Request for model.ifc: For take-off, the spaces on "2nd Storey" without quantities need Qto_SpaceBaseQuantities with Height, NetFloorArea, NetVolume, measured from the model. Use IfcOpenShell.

First a look at what the model holds.

```python
import ifcopenshell
import ifcopenshell.util.element
import ifcopenshell.util.unit

model = ifcopenshell.open("model.ifc")
print(model.schema)
for unit_type in ("LENGTHUNIT", "AREAUNIT", "VOLUMEUNIT"):
    print(unit_type, ifcopenshell.util.unit.calculate_unit_scale(model, unit_type))
storey = next(s for s in model.by_type("IfcBuildingStorey") if s.Name == "2nd Storey")
spaces = [e for e in ifcopenshell.util.element.get_decomposition(storey) if e.is_a("IfcSpace")]
for e in sorted(spaces, key=lambda e: e.id()):
    print(e.id(), e.is_a(), e.Name, list(ifcopenshell.util.element.get_psets(e, qtos_only=True)), sep=" | ")
```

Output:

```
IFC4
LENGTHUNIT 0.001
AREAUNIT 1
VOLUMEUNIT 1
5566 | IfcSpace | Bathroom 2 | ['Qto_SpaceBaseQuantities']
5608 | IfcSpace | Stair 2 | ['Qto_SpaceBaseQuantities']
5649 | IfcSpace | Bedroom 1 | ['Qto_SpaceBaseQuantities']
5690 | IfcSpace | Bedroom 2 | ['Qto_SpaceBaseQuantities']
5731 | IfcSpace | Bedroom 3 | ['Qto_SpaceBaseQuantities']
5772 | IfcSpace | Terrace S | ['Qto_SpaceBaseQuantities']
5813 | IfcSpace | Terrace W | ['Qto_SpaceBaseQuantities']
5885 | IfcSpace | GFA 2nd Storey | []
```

```python
import ifcopenshell
import ifcopenshell.api.pset
import ifcopenshell.geom
import ifcopenshell.util.element
import ifcopenshell.util.shape
import ifcopenshell.util.unit

model = ifcopenshell.open("model.ifc")
unit_scale = ifcopenshell.util.unit.calculate_unit_scale(model)
area_scale = ifcopenshell.util.unit.calculate_unit_scale(model, "AREAUNIT")
volume_scale = ifcopenshell.util.unit.calculate_unit_scale(model, "VOLUMEUNIT")
settings = ifcopenshell.geom.settings()

storey = next(s for s in model.by_type("IfcBuildingStorey") if s.Name == "2nd Storey")
spaces = [e for e in ifcopenshell.util.element.get_decomposition(storey) if e.is_a("IfcSpace")]

for e in sorted(spaces, key=lambda e: e.id()):
    if ifcopenshell.util.element.get_psets(e, qtos_only=True, should_inherit=False):
        continue
    # Geometry comes back in metres, in the element's own axes.
    shape = ifcopenshell.geom.create_shape(settings, e)
    values = {
        "Height": ifcopenshell.util.shape.get_z(shape.geometry) / unit_scale,
        "NetFloorArea": ifcopenshell.util.shape.get_footprint_area(shape.geometry) / area_scale,
        "NetVolume": ifcopenshell.util.shape.get_volume(shape.geometry) / volume_scale,
    }
    qto = ifcopenshell.api.pset.add_qto(model, product=e, name="Qto_SpaceBaseQuantities")
    ifcopenshell.api.pset.edit_qto(model, qto=qto, properties=values)
    print(e.id(), {k: round(v, 3) for k, v in values.items()})

model.write("model_v2.ifc")
```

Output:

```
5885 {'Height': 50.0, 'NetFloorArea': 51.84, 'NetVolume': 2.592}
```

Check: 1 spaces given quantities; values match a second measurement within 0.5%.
